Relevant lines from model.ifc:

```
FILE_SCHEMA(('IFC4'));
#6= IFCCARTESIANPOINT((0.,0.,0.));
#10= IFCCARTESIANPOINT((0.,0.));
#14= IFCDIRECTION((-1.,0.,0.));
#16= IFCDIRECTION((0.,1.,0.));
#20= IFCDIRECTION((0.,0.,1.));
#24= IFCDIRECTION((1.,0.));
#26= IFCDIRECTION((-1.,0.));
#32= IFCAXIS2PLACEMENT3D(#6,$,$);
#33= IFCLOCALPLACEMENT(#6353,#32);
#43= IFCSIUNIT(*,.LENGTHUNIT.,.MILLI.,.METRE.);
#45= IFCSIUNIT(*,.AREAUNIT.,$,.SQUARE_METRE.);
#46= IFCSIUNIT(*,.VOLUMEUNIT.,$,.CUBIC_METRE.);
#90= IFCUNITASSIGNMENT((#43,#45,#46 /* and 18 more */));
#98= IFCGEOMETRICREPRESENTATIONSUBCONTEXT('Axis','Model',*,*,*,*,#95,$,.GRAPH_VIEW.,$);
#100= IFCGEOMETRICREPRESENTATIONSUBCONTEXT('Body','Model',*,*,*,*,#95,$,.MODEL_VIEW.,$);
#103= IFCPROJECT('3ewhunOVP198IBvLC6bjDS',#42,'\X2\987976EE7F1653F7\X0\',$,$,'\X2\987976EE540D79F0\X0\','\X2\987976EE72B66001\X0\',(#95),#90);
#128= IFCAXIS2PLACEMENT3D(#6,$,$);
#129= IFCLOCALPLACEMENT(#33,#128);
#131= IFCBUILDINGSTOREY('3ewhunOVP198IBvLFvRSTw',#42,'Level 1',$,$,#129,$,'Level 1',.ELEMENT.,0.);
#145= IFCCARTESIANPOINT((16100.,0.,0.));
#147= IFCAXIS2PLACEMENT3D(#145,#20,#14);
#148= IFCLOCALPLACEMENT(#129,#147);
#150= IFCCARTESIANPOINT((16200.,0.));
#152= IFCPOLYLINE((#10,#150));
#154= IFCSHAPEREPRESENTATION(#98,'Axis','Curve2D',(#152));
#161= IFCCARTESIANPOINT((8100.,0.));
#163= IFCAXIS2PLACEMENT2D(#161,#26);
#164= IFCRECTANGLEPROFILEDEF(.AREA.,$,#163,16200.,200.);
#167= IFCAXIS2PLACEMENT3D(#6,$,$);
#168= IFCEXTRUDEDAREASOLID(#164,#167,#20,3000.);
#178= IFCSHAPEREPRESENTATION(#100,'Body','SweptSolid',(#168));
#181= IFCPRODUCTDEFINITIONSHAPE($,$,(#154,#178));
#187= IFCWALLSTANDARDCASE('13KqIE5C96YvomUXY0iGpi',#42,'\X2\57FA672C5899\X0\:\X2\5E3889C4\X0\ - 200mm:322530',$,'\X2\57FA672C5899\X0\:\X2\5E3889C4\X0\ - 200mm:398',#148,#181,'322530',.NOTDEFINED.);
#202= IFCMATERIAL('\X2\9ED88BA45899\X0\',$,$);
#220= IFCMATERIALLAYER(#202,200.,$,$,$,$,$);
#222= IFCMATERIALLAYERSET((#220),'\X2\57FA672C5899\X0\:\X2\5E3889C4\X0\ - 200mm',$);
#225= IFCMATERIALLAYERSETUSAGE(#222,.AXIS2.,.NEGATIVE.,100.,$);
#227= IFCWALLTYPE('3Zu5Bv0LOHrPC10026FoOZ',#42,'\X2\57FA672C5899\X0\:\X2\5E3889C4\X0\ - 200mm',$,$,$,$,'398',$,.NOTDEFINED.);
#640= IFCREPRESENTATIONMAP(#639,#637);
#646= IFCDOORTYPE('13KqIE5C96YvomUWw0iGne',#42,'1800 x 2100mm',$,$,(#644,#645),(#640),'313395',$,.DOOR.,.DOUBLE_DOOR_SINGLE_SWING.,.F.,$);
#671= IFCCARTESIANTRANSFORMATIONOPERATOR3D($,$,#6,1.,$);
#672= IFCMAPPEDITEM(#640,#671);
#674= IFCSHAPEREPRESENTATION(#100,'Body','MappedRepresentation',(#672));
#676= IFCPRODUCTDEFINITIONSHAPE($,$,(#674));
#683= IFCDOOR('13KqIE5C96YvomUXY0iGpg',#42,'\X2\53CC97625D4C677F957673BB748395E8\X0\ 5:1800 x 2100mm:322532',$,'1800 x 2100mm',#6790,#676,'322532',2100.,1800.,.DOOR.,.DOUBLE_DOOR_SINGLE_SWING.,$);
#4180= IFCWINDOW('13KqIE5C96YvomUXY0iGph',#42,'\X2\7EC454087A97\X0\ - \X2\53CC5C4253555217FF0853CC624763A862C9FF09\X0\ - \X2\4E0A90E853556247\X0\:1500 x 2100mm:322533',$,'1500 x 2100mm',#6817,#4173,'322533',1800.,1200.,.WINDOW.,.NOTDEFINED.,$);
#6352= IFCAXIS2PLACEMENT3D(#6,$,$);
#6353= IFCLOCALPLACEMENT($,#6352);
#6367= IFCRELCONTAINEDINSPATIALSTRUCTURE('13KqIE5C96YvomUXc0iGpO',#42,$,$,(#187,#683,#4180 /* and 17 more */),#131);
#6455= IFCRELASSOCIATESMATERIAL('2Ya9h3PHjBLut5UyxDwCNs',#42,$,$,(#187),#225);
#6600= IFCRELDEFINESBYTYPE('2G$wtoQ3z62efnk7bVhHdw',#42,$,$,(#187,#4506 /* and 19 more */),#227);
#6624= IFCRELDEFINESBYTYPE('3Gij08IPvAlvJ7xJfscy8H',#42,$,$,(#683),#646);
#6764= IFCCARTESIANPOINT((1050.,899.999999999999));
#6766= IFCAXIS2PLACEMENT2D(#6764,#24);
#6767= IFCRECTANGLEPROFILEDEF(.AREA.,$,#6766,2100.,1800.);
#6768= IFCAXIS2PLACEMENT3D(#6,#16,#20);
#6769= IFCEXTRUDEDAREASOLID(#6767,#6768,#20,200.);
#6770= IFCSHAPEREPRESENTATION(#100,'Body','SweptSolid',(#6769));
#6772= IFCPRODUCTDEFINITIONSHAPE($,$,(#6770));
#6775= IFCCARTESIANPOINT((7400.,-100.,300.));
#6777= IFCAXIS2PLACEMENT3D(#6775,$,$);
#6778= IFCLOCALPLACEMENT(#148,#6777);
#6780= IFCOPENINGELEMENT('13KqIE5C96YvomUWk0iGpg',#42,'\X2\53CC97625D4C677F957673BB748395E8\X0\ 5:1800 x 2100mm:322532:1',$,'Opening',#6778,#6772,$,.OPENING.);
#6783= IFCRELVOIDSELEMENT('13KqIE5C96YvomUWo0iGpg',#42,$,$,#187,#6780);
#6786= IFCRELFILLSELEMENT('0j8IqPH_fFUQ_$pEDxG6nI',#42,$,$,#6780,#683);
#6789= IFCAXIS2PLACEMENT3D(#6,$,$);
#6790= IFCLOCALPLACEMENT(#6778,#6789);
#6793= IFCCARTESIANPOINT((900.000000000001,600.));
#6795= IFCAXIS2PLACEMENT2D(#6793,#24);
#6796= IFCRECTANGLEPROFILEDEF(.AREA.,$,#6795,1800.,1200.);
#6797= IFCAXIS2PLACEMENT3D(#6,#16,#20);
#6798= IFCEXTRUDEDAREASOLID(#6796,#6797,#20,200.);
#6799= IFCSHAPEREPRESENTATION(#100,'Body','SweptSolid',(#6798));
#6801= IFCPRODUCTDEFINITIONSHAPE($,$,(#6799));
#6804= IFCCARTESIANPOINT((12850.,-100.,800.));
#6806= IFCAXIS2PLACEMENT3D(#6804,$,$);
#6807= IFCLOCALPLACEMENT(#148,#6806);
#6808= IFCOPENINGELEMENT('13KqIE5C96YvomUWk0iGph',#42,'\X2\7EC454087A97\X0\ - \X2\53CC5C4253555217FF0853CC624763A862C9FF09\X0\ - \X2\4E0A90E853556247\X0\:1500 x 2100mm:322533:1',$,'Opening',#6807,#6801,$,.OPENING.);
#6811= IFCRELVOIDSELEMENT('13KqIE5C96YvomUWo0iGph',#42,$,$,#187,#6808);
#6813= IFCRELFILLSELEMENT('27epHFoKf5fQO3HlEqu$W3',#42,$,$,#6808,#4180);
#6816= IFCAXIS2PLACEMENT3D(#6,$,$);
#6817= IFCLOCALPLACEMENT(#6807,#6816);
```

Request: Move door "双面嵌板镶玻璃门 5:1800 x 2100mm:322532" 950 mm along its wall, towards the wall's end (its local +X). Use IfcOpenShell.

```python
import ifcopenshell
import ifcopenshell.api.geometry
import ifcopenshell.util.placement

model = ifcopenshell.open("model.ifc")

door = model.by_guid("13KqIE5C96YvomUXY0iGpg")
opening = door.FillsVoids[0].RelatingOpeningElement
wall = opening.VoidsElements[0].RelatingBuildingElement

wall_matrix = ifcopenshell.util.placement.get_local_placement(wall.ObjectPlacement)
shift = wall_matrix[:3, 0] * 950.0
before = ifcopenshell.util.placement.get_local_placement(door.ObjectPlacement)[:3, 3].copy()

# The door is placed relative to its opening, so it follows when the opening moves.
matrix = ifcopenshell.util.placement.get_local_placement(opening.ObjectPlacement)
matrix[:3, 3] += shift
ifcopenshell.api.geometry.edit_object_placement(
    model, product=opening, matrix=matrix, is_si=False, should_transform_children=True
)

after = ifcopenshell.util.placement.get_local_placement(door.ObjectPlacement)[:3, 3]
print("door moved by", (after - before).round(3) + 0.0)

model.write("model_edited.ifc")
```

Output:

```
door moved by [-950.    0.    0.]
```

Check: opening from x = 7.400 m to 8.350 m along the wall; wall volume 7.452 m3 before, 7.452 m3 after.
